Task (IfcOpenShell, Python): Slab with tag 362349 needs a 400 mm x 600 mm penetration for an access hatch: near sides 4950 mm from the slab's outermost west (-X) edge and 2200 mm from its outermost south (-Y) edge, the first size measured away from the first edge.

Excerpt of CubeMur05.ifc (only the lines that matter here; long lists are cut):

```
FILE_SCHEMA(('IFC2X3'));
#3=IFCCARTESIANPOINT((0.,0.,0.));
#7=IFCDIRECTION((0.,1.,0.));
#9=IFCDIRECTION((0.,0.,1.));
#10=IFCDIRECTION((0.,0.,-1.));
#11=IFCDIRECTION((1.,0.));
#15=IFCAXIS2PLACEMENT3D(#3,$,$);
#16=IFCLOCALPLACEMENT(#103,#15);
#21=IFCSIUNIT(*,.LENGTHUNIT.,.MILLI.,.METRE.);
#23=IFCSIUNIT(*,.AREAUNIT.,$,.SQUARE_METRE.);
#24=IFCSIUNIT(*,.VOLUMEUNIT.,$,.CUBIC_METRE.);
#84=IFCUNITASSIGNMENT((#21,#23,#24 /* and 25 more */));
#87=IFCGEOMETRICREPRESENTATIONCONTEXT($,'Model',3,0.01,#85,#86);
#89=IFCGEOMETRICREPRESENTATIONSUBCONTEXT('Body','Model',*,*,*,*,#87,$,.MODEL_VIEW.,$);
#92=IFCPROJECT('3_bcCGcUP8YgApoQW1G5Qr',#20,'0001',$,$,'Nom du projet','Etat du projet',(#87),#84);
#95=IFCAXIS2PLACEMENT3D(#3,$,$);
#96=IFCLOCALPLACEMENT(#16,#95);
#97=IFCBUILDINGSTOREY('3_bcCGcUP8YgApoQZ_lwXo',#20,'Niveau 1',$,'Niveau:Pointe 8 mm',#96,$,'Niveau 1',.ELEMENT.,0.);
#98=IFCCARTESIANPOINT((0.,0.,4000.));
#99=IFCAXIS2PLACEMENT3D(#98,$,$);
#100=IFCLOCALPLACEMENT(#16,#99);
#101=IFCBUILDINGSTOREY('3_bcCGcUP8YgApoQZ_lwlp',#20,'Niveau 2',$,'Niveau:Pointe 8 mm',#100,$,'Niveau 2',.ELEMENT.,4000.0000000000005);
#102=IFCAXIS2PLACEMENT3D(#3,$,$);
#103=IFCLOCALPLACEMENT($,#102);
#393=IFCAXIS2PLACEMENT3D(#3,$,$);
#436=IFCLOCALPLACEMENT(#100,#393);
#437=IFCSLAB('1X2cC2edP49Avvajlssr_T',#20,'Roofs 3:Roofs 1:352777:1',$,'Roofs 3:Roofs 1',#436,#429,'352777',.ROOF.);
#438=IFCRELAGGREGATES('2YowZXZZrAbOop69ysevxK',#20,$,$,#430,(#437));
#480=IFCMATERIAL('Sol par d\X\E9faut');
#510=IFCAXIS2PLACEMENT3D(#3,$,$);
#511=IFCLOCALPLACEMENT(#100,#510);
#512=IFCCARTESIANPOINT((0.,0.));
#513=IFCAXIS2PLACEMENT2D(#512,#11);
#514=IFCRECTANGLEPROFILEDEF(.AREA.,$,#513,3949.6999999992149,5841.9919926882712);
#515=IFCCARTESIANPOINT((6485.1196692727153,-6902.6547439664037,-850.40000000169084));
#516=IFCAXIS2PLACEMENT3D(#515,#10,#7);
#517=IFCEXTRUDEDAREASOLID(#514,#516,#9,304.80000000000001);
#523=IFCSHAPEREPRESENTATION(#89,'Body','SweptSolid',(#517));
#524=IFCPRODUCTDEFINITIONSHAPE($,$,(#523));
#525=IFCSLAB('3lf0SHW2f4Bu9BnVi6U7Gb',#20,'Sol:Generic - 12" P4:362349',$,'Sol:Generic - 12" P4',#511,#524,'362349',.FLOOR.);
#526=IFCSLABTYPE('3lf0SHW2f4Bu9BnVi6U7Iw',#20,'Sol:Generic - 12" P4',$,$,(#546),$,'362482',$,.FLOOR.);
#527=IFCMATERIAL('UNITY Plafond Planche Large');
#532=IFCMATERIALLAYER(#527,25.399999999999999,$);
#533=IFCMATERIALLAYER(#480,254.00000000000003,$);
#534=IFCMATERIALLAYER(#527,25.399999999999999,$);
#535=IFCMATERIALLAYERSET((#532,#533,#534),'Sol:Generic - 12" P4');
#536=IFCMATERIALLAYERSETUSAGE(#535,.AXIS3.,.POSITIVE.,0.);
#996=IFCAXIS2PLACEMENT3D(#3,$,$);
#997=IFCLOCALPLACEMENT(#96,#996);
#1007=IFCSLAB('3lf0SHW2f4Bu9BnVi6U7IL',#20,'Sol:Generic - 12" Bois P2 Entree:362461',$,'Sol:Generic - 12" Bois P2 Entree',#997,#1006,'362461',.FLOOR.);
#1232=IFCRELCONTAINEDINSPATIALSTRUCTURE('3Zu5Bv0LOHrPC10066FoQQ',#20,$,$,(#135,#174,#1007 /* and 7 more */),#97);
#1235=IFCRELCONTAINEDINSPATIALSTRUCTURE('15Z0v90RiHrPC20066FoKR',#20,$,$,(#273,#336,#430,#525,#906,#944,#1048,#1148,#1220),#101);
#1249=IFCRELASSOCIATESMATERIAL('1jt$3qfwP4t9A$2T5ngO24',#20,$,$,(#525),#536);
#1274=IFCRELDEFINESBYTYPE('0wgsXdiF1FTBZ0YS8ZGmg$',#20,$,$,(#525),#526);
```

```python
import numpy as np
import ifcopenshell
import ifcopenshell.api.feature
import ifcopenshell.api.geometry
import ifcopenshell.api.root
import ifcopenshell.geom
import ifcopenshell.util.placement
import ifcopenshell.util.representation
import ifcopenshell.util.shape
import ifcopenshell.util.unit

model = ifcopenshell.open("CubeMur05.ifc")
unit_scale = ifcopenshell.util.unit.calculate_unit_scale(model)
settings = ifcopenshell.geom.settings()


def volume(element):
    """Net volume in cubic metres, openings subtracted."""
    shape = ifcopenshell.geom.create_shape(settings, element)
    return ifcopenshell.util.shape.get_volume(shape.geometry)


slab = model.by_guid("3lf0SHW2f4Bu9BnVi6U7Gb")
before = volume(slab)

# Extent in the slab's own axes, in metres. The edges named are its -X and -Y sides.
slab_shape = ifcopenshell.geom.create_shape(settings, slab)
vertices = ifcopenshell.util.shape.get_vertices(slab_shape.geometry)
x_min, y_min, bottom = vertices.min(axis=0)
top = vertices[:, 2].max()

opening = ifcopenshell.api.root.create_entity(model, ifc_class="IfcOpeningElement", name="Access hatch opening")
context = ifcopenshell.util.representation.get_context(model, "Model", "Body", "MODEL_VIEW")
width, depth = 0.4, 0.6
outline = [(0.0, 0.0), (width, 0.0), (width, depth), (0.0, depth), (0.0, 0.0)]
# Overshoot both faces by 50 mm so the cut is clean.
shape = ifcopenshell.api.geometry.add_slab_representation(
    model, context=context, depth=top - bottom + 0.1, polyline=outline
)
ifcopenshell.api.geometry.assign_representation(model, product=opening, representation=shape)

matrix = ifcopenshell.util.placement.get_local_placement(slab.ObjectPlacement)
matrix[:, 3] = matrix @ np.append(np.array([x_min + 4.95, y_min + 2.2, bottom - 0.05]) / unit_scale, 1.0)
ifcopenshell.api.geometry.edit_object_placement(model, product=opening, matrix=matrix, is_si=False)
ifcopenshell.api.feature.add_feature(model, feature=opening, element=slab)

after = volume(slab)

print(f"slab volume {before:.3f} -> {after:.3f} m3")

model.write("CubeMur05_rev.ifc")
```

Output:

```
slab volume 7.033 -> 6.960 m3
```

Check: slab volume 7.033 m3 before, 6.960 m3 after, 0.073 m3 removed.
